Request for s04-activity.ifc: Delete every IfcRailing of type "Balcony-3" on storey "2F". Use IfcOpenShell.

First a look at what the model holds.

```python
import ifcopenshell
import ifcopenshell.util.element

model = ifcopenshell.open("s04-activity.ifc")
print(model.schema)
storey = next(s for s in model.by_type("IfcBuildingStorey") if s.Name == "2F")
railings = [e for e in ifcopenshell.util.element.get_decomposition(storey) if e.is_a("IfcRailing")]
seen = {}
for e in railings:
    element_type = ifcopenshell.util.element.get_type(e)
    name = element_type.Name if element_type not in (None, e) else None
    seen[name] = seen.get(name, 0) + 1
for name, count in sorted(seen.items(), key=str):
    print(count, "x", name)
```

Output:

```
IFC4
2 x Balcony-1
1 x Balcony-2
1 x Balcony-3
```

```python
import ifcopenshell
import ifcopenshell.api.root
import ifcopenshell.util.element

model = ifcopenshell.open("s04-activity.ifc")

storey = next(s for s in model.by_type("IfcBuildingStorey") if s.Name == "2F")
railings = [e for e in ifcopenshell.util.element.get_decomposition(storey) if e.is_a("IfcRailing")]
targets = [e for e in railings if (t := ifcopenshell.util.element.get_type(e)) not in (None, e) and t.Name == "Balcony-3"]

for e in targets:
    ifcopenshell.api.root.remove_product(model, product=e)
print(len(targets), "removed")

model.write("s04-activity_v2.ifc")
```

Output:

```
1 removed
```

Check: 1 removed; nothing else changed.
